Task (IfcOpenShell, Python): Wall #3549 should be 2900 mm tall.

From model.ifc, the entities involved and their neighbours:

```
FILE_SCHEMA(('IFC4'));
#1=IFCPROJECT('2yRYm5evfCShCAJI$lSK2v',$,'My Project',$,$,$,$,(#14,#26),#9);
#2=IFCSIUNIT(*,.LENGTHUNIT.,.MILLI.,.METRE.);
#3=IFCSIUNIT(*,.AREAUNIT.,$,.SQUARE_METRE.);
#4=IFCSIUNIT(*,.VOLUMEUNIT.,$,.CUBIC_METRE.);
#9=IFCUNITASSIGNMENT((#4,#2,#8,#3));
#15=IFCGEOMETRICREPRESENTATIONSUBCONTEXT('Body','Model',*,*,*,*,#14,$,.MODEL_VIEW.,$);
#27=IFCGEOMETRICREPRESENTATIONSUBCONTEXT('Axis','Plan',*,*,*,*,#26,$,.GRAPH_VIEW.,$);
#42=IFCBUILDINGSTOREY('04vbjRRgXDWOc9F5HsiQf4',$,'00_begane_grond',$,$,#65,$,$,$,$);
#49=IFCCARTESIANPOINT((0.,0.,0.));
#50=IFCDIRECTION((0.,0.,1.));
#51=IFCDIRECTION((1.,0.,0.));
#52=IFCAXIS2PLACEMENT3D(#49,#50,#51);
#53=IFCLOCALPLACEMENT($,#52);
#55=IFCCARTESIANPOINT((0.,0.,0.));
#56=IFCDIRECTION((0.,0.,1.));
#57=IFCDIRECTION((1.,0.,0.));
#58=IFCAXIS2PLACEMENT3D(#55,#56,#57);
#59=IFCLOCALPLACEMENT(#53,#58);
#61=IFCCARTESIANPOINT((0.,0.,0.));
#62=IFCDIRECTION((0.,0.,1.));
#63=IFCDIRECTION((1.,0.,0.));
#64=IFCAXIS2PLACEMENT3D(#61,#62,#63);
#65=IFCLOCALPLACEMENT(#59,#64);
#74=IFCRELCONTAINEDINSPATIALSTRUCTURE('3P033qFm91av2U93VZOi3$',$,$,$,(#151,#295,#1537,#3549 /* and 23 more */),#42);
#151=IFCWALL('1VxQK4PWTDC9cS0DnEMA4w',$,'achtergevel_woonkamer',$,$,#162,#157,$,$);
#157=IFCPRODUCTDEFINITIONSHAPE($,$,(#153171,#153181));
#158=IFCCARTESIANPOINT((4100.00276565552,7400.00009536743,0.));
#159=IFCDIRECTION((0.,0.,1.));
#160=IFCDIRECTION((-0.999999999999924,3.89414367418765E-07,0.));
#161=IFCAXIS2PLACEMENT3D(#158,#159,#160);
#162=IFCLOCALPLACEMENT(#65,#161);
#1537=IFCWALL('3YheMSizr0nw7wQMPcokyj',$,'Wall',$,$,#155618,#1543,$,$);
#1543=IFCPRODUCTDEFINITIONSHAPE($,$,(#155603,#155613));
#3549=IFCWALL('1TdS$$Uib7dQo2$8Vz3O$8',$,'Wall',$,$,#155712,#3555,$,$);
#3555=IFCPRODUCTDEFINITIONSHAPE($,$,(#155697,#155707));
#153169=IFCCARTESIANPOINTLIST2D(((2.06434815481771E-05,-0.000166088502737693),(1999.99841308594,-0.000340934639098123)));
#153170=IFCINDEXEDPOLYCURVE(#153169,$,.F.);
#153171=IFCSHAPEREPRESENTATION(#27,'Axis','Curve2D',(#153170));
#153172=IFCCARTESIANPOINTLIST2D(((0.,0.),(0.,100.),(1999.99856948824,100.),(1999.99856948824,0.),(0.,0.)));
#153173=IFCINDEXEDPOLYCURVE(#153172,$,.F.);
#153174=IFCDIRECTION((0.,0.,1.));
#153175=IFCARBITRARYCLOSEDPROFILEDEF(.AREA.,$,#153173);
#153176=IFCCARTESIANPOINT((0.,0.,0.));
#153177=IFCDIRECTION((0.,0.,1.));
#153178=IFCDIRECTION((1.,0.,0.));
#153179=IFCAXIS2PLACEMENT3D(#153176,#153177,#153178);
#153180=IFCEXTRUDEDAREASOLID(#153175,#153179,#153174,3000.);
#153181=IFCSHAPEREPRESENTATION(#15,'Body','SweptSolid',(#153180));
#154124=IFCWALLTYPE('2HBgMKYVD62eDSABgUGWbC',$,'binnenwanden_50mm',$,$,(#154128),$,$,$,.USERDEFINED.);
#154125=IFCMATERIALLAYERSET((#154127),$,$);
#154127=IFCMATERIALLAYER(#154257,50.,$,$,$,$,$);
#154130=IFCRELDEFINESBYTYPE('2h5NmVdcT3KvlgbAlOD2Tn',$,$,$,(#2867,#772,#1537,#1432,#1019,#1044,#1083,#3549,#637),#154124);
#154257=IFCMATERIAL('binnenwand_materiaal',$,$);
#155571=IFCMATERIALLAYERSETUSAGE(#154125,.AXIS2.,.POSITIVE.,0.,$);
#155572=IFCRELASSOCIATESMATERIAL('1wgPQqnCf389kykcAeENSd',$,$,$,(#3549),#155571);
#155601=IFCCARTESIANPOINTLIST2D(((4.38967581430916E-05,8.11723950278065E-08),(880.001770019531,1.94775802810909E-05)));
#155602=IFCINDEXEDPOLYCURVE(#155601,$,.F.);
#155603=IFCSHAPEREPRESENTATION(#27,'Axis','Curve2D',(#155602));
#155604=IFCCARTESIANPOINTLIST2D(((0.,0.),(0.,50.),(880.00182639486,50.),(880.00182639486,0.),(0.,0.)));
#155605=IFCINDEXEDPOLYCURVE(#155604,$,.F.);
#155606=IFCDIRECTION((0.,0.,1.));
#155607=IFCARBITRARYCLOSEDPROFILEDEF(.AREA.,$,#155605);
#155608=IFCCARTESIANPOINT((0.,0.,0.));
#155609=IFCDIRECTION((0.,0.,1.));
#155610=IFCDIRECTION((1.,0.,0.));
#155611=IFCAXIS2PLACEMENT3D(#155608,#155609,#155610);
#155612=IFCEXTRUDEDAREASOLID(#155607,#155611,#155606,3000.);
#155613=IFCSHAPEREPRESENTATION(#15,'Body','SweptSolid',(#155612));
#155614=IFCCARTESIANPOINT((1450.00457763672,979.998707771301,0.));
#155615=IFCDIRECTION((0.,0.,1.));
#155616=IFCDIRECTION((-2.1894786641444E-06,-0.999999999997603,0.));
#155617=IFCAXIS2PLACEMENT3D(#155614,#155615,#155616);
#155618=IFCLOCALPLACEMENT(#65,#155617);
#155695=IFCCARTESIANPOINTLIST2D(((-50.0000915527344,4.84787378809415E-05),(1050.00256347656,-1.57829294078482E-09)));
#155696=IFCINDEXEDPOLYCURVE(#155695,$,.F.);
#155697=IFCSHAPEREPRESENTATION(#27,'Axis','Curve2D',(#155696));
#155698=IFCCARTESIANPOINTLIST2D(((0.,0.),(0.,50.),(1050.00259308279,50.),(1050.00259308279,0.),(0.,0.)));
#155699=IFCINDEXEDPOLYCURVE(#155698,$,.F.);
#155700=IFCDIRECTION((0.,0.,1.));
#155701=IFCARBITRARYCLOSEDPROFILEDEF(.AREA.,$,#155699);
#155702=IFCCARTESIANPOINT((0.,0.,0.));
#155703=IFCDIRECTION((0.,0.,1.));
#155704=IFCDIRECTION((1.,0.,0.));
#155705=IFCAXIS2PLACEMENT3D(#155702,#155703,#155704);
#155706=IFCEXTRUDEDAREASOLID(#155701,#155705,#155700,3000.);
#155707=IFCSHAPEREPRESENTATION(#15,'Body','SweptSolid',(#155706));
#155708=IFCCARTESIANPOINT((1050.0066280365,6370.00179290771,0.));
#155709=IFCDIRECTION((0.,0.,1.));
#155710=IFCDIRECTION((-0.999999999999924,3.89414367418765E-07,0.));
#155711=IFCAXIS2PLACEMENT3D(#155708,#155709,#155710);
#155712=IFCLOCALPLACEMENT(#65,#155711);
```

```python
import ifcopenshell
import ifcopenshell.geom
import ifcopenshell.util.representation
import ifcopenshell.util.shape

model = ifcopenshell.open("model.ifc")
settings = ifcopenshell.geom.settings()


def volume(element):
    """Net volume in cubic metres, openings subtracted."""
    shape = ifcopenshell.geom.create_shape(settings, element)
    return ifcopenshell.util.shape.get_volume(shape.geometry)


wall = model.by_id(3549)
before = volume(wall)

body = ifcopenshell.util.representation.get_representation(wall, "Model", "Body")
solid = body.Items[0]
old_height = solid.Depth
solid.Depth = 2900.0
after = volume(wall)

print(f"height {old_height:g} -> {solid.Depth:g}, volume {before:.3f} -> {after:.3f} m3")

model.write("model_rev.ifc")
```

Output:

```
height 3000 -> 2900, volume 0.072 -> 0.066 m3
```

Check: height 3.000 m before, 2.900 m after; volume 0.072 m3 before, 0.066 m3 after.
